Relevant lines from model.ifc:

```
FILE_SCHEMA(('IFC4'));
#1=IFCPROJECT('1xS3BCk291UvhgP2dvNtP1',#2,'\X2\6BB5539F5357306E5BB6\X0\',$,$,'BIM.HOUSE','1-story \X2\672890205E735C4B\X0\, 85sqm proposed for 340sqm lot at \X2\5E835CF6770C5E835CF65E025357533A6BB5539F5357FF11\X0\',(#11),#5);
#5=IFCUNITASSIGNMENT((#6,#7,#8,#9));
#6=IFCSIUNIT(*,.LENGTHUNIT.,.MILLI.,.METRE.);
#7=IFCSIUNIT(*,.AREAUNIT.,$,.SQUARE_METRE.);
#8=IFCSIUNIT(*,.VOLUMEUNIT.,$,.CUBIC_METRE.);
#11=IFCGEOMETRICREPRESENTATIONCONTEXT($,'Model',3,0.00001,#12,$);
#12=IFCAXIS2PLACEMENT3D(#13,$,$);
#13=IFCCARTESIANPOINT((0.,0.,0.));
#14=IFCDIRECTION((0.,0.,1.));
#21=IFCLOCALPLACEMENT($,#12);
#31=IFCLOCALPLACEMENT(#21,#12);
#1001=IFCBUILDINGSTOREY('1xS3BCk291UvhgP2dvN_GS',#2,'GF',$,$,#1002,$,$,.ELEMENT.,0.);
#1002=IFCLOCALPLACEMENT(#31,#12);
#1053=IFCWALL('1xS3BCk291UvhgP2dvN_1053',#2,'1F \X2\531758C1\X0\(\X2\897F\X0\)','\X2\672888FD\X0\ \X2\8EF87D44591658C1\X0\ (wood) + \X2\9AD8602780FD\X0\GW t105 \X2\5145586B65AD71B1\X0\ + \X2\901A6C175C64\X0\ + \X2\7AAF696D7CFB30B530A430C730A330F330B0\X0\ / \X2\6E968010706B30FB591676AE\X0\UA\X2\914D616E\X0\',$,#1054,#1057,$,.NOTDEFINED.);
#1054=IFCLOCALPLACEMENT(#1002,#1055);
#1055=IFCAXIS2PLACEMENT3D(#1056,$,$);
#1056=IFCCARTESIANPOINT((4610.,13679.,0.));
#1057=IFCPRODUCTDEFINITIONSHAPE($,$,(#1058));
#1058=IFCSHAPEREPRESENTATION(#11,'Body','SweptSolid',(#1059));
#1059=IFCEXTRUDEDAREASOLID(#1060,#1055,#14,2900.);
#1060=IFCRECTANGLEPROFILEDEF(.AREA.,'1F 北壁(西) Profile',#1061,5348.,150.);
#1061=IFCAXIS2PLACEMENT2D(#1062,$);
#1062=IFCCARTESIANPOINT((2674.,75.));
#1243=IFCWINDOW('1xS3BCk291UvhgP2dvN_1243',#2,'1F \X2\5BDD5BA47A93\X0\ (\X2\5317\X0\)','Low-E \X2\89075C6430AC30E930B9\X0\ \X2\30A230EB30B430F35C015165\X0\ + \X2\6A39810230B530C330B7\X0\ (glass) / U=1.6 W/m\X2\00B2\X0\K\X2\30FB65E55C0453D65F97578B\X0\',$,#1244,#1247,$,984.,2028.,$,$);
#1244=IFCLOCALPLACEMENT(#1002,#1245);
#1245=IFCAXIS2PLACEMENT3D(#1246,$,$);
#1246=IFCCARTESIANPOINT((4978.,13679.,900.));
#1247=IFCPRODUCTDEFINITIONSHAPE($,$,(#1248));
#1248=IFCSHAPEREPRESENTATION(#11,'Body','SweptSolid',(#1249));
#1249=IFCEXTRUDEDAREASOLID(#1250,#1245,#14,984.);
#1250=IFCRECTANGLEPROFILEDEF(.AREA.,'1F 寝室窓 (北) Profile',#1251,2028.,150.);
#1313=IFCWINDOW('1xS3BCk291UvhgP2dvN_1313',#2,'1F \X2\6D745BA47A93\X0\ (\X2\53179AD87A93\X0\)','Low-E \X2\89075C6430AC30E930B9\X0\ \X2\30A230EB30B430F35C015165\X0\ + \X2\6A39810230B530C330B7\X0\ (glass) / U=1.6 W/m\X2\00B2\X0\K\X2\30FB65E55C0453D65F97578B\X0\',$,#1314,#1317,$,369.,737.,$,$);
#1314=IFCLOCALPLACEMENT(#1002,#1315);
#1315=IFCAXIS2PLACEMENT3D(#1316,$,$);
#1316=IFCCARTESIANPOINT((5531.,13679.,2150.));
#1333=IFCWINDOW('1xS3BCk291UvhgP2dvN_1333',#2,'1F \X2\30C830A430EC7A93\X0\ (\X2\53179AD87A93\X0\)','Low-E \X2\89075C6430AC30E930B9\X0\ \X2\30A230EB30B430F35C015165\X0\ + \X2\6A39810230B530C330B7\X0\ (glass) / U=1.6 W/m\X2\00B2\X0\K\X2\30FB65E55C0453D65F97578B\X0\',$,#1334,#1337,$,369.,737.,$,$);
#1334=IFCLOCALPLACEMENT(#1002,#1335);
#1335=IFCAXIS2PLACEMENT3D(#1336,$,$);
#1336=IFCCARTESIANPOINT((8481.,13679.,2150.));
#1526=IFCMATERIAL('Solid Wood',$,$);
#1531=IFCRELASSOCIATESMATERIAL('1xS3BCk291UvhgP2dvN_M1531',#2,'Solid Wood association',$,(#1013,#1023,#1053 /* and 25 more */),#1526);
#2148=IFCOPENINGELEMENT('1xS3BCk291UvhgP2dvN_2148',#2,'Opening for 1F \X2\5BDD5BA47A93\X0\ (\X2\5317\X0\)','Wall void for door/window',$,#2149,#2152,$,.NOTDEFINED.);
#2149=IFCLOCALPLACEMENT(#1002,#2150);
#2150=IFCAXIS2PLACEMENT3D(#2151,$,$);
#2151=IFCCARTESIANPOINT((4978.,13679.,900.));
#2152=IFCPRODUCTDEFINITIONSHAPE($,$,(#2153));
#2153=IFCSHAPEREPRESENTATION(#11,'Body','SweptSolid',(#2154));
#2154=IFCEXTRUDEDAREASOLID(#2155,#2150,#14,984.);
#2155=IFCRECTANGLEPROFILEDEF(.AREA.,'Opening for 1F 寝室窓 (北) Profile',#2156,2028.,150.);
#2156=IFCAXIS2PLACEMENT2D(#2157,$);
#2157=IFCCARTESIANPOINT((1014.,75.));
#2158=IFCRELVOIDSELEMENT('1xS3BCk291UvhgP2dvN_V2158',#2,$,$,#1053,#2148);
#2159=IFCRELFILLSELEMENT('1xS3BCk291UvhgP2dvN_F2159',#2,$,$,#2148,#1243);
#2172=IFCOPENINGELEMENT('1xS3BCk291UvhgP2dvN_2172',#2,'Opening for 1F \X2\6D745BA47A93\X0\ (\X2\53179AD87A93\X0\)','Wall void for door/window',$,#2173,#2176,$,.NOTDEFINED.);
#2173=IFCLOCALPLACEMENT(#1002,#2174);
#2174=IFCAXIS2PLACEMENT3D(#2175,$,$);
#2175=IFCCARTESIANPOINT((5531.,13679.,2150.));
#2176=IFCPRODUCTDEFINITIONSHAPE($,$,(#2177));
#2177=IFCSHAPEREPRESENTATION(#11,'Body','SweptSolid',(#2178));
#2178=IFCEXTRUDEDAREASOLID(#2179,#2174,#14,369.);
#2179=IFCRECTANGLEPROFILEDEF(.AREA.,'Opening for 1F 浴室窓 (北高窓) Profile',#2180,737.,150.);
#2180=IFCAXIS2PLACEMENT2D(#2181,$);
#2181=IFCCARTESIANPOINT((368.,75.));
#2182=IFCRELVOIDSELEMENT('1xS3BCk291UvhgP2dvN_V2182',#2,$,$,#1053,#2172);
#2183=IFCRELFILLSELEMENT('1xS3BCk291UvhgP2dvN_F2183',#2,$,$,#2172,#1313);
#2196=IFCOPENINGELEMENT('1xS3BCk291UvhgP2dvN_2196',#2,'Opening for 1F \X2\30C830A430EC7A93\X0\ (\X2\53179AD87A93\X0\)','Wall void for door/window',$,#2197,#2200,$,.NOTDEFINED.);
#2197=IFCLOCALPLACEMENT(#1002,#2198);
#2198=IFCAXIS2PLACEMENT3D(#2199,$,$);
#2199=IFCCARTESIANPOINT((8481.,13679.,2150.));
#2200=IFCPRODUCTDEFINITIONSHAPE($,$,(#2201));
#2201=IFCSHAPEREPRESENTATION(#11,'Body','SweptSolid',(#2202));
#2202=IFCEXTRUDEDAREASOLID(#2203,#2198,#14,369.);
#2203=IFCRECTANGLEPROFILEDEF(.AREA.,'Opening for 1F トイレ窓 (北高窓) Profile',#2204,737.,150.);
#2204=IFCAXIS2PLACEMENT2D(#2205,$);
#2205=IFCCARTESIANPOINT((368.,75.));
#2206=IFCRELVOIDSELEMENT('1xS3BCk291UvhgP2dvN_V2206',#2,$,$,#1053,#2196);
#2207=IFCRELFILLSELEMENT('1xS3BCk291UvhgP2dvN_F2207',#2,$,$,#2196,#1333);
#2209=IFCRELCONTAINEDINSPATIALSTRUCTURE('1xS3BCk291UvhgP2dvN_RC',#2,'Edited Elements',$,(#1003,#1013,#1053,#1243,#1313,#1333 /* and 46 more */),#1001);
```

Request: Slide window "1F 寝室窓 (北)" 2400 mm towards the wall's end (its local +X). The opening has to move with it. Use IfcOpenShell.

```python
import ifcopenshell
import ifcopenshell.api.geometry
import ifcopenshell.util.placement
import ifcopenshell.util.unit

model = ifcopenshell.open("model.ifc")
unit_scale = ifcopenshell.util.unit.calculate_unit_scale(model)

window = model.by_id(1243)
opening = window.FillsVoids[0].RelatingOpeningElement
wall = opening.VoidsElements[0].RelatingBuildingElement

wall_matrix = ifcopenshell.util.placement.get_local_placement(wall.ObjectPlacement)
shift = wall_matrix[:3, 0] * 2.4 / unit_scale
before = ifcopenshell.util.placement.get_local_placement(window.ObjectPlacement)[:3, 3].copy()

# The window is not placed relative to its opening, so move both.
for product in (opening, window):
    matrix = ifcopenshell.util.placement.get_local_placement(product.ObjectPlacement)
    matrix[:3, 3] += shift
    ifcopenshell.api.geometry.edit_object_placement(model, product=product, matrix=matrix, is_si=False)

after = ifcopenshell.util.placement.get_local_placement(window.ObjectPlacement)[:3, 3]
print("window moved by", (after - before).round(3) + 0.0)

model.write("model_updated.ifc")
```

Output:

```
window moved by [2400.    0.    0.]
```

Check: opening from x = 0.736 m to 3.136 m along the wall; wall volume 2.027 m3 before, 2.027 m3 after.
